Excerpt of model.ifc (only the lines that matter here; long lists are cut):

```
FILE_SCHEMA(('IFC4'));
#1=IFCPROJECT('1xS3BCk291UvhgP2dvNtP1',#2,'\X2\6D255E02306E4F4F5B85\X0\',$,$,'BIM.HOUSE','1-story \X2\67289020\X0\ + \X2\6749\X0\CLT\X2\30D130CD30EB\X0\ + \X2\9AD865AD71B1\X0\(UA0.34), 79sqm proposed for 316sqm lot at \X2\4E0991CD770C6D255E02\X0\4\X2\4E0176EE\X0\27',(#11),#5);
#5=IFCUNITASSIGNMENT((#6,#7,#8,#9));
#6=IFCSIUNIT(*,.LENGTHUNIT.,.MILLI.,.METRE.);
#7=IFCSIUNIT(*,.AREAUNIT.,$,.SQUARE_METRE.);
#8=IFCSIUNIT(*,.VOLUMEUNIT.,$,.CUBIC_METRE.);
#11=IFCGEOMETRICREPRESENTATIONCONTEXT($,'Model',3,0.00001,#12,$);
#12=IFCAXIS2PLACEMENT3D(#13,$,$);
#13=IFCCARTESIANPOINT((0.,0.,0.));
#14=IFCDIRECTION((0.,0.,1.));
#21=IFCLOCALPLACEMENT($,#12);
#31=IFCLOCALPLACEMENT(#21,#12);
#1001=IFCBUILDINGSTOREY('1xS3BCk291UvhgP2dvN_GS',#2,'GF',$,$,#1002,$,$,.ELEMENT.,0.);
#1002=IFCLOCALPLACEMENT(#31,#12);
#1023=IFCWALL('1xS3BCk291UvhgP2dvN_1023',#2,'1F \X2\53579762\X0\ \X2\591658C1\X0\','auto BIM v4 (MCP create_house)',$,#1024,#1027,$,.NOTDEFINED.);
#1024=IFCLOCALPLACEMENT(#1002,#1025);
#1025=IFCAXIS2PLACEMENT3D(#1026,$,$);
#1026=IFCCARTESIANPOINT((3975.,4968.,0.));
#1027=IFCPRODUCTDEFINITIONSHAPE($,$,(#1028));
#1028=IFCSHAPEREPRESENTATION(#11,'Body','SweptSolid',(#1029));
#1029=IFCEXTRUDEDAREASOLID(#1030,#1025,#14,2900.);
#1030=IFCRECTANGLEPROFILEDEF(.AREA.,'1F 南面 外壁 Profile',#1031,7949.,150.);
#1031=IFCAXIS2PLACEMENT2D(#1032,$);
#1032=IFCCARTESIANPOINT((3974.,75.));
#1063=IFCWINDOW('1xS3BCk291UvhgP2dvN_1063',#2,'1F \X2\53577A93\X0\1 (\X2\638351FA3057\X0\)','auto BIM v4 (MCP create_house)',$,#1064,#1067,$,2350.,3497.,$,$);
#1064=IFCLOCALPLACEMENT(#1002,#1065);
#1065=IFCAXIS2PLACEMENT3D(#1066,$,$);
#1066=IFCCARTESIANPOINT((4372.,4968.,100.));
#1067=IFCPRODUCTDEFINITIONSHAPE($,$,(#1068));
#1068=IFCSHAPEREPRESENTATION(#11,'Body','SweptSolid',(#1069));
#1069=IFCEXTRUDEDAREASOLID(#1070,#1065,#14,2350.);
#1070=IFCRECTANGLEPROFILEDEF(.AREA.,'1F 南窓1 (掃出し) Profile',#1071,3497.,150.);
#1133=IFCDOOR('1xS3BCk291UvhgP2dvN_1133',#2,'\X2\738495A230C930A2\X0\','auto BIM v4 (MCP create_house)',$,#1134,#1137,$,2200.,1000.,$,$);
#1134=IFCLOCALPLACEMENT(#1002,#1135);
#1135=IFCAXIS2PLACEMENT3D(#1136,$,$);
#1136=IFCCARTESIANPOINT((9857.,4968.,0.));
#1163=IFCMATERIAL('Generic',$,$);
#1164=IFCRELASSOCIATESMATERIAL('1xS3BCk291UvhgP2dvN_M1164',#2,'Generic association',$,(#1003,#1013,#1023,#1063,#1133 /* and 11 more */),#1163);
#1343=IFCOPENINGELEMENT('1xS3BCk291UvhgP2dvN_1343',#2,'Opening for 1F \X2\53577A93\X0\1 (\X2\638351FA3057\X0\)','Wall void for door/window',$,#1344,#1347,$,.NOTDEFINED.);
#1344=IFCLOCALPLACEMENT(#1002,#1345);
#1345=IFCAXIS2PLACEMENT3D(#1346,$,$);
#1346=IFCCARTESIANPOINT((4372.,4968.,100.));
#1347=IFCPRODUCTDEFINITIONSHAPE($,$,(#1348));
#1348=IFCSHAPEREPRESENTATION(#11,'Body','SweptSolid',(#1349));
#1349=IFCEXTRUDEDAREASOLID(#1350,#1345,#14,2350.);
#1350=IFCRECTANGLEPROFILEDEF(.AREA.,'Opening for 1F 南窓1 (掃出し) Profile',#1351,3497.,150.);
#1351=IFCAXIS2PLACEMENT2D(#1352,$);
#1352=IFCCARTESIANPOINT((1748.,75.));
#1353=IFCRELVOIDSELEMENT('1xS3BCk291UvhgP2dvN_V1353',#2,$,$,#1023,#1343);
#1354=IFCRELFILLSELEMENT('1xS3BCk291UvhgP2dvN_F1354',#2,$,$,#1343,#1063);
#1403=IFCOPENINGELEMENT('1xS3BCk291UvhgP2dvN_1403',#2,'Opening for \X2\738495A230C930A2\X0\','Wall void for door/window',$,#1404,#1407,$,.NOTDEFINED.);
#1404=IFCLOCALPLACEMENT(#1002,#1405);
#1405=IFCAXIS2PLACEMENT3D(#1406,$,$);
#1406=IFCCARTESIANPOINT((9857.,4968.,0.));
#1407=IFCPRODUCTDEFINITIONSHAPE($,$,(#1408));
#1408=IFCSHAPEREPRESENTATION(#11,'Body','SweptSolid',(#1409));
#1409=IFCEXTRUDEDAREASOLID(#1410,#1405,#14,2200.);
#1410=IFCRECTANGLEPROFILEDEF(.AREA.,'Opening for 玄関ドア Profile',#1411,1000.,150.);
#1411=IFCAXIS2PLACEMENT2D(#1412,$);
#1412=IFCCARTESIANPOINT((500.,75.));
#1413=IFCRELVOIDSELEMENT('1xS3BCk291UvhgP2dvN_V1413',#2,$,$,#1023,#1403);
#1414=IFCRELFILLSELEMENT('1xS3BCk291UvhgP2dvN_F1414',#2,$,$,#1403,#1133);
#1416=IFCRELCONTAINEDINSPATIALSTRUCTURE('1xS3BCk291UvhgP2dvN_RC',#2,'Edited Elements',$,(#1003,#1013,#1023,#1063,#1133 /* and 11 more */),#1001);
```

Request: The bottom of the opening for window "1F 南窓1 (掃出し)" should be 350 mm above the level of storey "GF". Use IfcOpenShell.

```python
import numpy as np
import ifcopenshell
import ifcopenshell.api.geometry
import ifcopenshell.geom
import ifcopenshell.util.element
import ifcopenshell.util.placement
import ifcopenshell.util.shape
import ifcopenshell.util.unit

model = ifcopenshell.open("model.ifc")
unit_scale = ifcopenshell.util.unit.calculate_unit_scale(model)

window = model.by_guid("1xS3BCk291UvhgP2dvN_1063")
opening = window.FillsVoids[0].RelatingOpeningElement
storey = ifcopenshell.util.element.get_container(window, ifc_class="IfcBuildingStorey")
level = ifcopenshell.util.placement.get_local_placement(storey.ObjectPlacement)[2, 3]

# The opening's origin need not be at the sill, so measure its lowest point.
shape = ifcopenshell.geom.create_shape(ifcopenshell.geom.settings(), opening)
bottom = ifcopenshell.util.shape.get_shape_bottom_elevation(shape, shape.geometry) / unit_scale
dz = level + 350.0 - bottom

shift = np.array([0.0, 0.0, dz])
# The window is not placed relative to its opening, so move both.
for product in (opening, window):
    matrix = ifcopenshell.util.placement.get_local_placement(product.ObjectPlacement)
    matrix[:3, 3] += shift
    ifcopenshell.api.geometry.edit_object_placement(model, product=product, matrix=matrix, is_si=False)

print(f"moved by {dz * unit_scale:+.3f} m")

model.write("model_rev.ifc")
```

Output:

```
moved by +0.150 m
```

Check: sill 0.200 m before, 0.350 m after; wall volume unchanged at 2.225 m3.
